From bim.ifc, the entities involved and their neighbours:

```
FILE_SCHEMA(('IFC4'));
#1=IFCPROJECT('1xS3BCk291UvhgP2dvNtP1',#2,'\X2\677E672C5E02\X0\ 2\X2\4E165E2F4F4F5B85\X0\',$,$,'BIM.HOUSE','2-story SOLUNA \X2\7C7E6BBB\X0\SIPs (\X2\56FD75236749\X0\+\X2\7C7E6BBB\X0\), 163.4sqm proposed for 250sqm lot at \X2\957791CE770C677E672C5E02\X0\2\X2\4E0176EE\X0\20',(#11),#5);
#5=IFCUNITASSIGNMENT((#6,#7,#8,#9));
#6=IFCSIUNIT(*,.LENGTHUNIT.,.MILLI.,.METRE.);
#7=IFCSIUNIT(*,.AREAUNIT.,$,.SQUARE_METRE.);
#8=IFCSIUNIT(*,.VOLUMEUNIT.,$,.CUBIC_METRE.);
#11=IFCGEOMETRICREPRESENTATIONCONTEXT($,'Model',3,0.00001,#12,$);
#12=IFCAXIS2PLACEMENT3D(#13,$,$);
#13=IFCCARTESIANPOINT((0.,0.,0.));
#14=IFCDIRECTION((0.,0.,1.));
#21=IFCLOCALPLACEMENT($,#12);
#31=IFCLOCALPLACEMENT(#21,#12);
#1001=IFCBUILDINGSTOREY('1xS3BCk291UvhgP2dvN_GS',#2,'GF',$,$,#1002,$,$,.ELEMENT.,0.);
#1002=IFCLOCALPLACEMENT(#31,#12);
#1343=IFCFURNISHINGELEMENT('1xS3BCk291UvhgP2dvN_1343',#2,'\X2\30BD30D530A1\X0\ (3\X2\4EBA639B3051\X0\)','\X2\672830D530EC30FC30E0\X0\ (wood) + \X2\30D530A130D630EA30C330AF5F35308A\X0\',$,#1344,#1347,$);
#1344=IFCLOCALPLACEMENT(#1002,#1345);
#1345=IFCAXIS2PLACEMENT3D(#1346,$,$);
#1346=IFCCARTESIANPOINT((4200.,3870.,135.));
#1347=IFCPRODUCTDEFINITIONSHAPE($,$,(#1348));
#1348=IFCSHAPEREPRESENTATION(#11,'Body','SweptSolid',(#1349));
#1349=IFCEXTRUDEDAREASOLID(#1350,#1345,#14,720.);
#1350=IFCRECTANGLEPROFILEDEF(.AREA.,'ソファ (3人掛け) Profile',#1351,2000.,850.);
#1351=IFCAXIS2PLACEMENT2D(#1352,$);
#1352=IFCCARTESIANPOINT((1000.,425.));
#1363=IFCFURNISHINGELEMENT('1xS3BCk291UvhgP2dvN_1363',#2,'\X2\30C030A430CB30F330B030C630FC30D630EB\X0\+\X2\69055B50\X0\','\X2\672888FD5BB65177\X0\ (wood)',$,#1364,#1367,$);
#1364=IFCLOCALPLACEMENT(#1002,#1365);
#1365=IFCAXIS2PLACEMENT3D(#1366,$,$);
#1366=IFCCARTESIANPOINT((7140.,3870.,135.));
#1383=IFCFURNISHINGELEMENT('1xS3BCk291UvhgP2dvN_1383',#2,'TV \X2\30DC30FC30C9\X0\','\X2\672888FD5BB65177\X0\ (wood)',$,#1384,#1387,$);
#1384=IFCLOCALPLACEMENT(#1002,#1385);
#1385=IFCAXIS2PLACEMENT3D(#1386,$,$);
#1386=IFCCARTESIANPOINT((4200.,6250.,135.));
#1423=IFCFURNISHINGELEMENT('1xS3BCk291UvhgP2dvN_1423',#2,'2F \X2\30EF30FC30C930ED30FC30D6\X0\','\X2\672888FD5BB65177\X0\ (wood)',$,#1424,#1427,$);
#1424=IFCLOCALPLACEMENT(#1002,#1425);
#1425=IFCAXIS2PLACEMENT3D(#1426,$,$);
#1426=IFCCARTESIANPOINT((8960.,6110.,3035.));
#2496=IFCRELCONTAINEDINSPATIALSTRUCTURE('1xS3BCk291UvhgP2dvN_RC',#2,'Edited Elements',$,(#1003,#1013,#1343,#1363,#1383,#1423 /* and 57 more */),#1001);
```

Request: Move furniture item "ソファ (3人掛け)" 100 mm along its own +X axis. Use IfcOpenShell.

```python
import ifcopenshell
import ifcopenshell.api.geometry
import ifcopenshell.util.placement
import ifcopenshell.util.unit

model = ifcopenshell.open("bim.ifc")
unit_scale = ifcopenshell.util.unit.calculate_unit_scale(model)

item = model.by_guid("1xS3BCk291UvhgP2dvN_1343")
matrix = ifcopenshell.util.placement.get_local_placement(item.ObjectPlacement)
matrix[:3, 3] += matrix[:3, 0] * 0.1 / unit_scale
ifcopenshell.api.geometry.edit_object_placement(model, product=item, matrix=matrix, is_si=False)

print(ifcopenshell.util.placement.get_local_placement(item.ObjectPlacement).round(3) + 0.0)

model.write("bim_rev.ifc")
```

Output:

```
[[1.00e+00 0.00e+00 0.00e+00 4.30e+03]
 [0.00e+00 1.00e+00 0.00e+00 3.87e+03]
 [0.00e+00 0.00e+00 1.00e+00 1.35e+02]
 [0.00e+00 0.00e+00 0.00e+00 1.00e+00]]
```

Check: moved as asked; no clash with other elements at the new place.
